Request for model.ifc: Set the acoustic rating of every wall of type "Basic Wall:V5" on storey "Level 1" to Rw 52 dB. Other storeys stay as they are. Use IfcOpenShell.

First a look at what the model holds.

```python
import ifcopenshell
import ifcopenshell.util.element

model = ifcopenshell.open("model.ifc")
print(model.schema)
storey = next(s for s in model.by_type("IfcBuildingStorey") if s.Name == "Level 1")
walls = [e for e in ifcopenshell.util.element.get_decomposition(storey) if e.is_a("IfcWall")]
seen = {}
for e in walls:
    element_type = ifcopenshell.util.element.get_type(e)
    key = (element_type.Name if element_type != e and element_type else None, ifcopenshell.util.element.get_pset(e, "Pset_WallCommon", "AcousticRating"))
    seen[key] = seen.get(key, 0) + 1
for (name, value), count in sorted(seen.items(), key=str):
    print(count, "x", name, "|", value)
```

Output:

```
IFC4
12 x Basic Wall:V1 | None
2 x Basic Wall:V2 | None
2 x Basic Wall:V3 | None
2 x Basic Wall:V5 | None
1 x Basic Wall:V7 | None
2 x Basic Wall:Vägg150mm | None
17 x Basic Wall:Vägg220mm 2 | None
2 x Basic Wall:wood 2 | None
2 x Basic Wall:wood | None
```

```python
import ifcopenshell
import ifcopenshell.api.pset
import ifcopenshell.util.element

model = ifcopenshell.open("model.ifc")

storey = next(s for s in model.by_type("IfcBuildingStorey") if s.Name == "Level 1")
walls = [e for e in ifcopenshell.util.element.get_decomposition(storey) if e.is_a("IfcWall")]

count = 0
for e in walls:
    element_type = ifcopenshell.util.element.get_type(e)
    if element_type in (None, e) or element_type.Name != "Basic Wall:V5":
        continue
    # add_pset returns the element's existing set when there is one.
    pset = ifcopenshell.api.pset.add_pset(model, product=e, name="Pset_WallCommon")
    ifcopenshell.api.pset.edit_pset(model, pset=pset, properties={"AcousticRating": "Rw 52 dB"})
    count += 1

print(count, "walls updated")

model.write("model_updated.ifc")
```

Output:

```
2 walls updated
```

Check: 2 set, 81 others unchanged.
